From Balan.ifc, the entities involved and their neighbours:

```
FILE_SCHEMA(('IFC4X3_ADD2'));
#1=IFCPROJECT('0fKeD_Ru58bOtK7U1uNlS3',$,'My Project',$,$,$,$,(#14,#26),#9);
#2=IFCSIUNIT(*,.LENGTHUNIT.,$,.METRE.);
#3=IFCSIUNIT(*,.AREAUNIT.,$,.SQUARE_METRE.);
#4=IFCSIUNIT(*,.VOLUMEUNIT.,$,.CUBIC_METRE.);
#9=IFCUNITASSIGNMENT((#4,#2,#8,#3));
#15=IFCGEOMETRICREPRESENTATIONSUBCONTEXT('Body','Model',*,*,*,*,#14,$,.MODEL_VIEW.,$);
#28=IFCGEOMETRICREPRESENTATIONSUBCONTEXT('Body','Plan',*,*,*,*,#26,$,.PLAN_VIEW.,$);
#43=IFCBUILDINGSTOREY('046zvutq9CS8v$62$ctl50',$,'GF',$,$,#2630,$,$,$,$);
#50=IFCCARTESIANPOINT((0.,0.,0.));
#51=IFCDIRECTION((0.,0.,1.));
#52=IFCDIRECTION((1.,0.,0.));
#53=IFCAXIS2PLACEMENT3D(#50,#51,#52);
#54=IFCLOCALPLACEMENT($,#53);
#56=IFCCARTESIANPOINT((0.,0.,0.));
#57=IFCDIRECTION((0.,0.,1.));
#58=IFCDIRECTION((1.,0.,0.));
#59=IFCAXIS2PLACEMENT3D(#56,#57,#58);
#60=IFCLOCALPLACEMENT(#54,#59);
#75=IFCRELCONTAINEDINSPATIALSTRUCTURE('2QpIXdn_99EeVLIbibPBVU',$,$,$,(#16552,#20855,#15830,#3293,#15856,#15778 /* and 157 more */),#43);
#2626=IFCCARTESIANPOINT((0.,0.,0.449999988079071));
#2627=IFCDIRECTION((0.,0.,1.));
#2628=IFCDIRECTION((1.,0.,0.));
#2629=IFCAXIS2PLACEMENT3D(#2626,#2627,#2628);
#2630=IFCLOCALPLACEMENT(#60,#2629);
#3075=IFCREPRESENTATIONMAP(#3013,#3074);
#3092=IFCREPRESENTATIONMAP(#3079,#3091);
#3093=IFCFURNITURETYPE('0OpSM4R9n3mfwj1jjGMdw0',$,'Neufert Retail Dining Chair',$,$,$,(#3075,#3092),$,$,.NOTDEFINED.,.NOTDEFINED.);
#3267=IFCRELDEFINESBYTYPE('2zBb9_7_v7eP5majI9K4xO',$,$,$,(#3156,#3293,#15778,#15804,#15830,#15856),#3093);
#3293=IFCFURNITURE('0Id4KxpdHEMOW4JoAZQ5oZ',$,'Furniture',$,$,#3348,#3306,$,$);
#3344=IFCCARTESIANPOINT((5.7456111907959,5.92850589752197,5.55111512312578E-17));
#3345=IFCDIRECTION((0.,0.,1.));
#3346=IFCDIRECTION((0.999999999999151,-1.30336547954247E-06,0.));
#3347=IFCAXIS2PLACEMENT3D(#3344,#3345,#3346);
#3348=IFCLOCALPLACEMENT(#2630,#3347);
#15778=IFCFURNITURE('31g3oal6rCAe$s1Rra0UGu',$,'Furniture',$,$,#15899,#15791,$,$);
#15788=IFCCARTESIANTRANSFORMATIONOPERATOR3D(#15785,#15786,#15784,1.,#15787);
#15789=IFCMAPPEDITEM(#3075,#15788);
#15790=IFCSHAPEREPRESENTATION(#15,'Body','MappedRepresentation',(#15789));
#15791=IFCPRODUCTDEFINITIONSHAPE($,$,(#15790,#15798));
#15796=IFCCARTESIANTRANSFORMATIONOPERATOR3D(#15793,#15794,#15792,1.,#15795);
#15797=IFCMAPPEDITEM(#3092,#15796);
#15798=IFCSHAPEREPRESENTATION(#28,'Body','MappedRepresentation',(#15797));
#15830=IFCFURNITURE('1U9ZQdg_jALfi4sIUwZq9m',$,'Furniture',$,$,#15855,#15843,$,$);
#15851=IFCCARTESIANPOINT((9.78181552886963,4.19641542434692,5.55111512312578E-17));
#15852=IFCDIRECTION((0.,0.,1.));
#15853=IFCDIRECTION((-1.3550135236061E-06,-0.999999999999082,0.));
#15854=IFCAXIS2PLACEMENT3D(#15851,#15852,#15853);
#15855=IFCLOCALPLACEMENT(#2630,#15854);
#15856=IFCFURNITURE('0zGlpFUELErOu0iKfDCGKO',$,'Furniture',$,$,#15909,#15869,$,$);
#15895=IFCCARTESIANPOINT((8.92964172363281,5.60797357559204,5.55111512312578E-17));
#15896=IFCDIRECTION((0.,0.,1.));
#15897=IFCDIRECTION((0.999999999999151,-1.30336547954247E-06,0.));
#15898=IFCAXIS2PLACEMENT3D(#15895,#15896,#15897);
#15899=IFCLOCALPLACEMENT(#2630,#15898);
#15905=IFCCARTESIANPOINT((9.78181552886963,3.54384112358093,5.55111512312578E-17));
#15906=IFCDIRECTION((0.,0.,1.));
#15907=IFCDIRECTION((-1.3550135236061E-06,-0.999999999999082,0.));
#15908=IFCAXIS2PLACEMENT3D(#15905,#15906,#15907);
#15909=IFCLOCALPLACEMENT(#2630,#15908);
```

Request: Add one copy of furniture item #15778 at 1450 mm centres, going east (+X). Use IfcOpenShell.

```python
import numpy as np
import ifcopenshell
import ifcopenshell.api.geometry
import ifcopenshell.api.root
import ifcopenshell.util.element
import ifcopenshell.util.placement
import ifcopenshell.util.unit

model = ifcopenshell.open("Balan.ifc")
unit_scale = ifcopenshell.util.unit.calculate_unit_scale(model)

source = model.by_guid("31g3oal6rCAe$s1Rra0UGu")
base = ifcopenshell.util.placement.get_local_placement(source.ObjectPlacement)
step = np.array([1.0, 0.0, 0.0]) * 1.45 / unit_scale

for i in range(1, 2):
    copy = ifcopenshell.api.root.copy_class(model, product=source)
    copy.Representation = ifcopenshell.util.element.copy_deep(
        model, source.Representation, exclude=["IfcGeometricRepresentationContext", "IfcRepresentationMap"]
    )
    matrix = base.copy()
    matrix[:3, 3] += i * step
    print("added at", matrix[:3, 3].round(3) + 0.0)
    ifcopenshell.api.geometry.edit_object_placement(model, product=copy, matrix=matrix, is_si=False)

model.write("Balan_rev.ifc")
```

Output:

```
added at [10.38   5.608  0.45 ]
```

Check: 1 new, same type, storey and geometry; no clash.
